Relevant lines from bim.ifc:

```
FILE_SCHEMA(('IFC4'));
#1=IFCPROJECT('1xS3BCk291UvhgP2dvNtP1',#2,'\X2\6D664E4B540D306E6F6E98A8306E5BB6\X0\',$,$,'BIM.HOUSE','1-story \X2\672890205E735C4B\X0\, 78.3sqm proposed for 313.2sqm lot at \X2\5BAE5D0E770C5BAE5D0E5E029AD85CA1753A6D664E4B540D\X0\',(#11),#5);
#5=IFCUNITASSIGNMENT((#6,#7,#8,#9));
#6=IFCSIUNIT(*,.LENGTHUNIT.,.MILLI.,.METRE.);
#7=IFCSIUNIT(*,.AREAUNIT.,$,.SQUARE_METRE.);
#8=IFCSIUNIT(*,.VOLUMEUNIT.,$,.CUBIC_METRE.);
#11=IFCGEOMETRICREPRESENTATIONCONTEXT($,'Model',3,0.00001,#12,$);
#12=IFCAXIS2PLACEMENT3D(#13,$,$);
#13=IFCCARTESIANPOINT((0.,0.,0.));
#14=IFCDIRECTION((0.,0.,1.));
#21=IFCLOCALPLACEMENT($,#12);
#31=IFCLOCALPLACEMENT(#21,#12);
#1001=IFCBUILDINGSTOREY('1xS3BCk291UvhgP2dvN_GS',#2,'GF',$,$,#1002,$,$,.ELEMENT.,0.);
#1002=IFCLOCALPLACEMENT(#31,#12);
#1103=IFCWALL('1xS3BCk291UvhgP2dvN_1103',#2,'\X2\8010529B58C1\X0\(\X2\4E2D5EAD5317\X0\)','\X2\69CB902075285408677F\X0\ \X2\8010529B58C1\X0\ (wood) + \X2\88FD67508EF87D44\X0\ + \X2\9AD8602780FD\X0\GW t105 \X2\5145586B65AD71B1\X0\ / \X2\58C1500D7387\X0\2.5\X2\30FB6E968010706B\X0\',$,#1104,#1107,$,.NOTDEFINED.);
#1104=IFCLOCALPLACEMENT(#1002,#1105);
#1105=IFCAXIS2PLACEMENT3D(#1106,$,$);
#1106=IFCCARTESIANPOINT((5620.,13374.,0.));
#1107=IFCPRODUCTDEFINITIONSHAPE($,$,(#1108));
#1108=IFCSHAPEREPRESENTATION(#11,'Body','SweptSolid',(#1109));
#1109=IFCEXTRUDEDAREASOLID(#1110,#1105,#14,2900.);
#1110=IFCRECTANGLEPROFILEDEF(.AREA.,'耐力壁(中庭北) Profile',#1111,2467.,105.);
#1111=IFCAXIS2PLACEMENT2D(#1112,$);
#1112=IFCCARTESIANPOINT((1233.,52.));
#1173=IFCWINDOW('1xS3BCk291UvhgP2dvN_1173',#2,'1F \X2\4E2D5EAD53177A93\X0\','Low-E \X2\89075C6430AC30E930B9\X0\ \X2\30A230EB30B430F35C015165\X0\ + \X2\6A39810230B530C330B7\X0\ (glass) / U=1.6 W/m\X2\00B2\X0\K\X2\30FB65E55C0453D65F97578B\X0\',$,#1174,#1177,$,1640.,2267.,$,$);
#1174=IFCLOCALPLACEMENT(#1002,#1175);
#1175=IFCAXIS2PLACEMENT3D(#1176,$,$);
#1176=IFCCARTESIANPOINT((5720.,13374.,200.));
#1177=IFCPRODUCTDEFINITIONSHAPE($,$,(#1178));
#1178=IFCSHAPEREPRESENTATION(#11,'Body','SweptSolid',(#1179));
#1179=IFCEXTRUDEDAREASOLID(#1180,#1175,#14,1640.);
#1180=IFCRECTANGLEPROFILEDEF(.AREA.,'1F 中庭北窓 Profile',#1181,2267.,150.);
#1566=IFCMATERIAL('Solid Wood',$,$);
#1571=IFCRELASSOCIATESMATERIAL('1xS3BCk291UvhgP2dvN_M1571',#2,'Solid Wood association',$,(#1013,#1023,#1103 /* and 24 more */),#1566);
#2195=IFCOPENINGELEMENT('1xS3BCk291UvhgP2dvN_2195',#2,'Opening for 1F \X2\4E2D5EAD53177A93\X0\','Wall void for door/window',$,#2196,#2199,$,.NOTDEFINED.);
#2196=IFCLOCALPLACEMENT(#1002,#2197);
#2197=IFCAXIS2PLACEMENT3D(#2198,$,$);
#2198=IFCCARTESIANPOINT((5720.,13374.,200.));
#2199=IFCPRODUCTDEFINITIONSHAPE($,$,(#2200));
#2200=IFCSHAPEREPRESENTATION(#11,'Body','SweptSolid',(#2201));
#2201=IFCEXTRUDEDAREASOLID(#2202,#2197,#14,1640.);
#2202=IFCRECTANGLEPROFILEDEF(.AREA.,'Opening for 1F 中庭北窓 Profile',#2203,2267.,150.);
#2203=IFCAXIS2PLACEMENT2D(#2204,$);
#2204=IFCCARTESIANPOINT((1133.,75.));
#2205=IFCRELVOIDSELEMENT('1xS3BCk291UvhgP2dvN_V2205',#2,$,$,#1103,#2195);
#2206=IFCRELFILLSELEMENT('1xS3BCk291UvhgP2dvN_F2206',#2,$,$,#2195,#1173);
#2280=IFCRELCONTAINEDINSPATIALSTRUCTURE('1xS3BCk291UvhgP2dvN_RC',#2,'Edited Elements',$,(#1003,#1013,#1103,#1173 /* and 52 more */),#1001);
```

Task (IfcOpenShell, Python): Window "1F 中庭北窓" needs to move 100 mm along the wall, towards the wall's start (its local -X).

```python
import ifcopenshell
import ifcopenshell.api.geometry
import ifcopenshell.util.placement

model = ifcopenshell.open("bim.ifc")

window = model.by_guid("1xS3BCk291UvhgP2dvN_1173")
opening = window.FillsVoids[0].RelatingOpeningElement
wall = opening.VoidsElements[0].RelatingBuildingElement

wall_matrix = ifcopenshell.util.placement.get_local_placement(wall.ObjectPlacement)
shift = wall_matrix[:3, 0] * -100.0
before = ifcopenshell.util.placement.get_local_placement(window.ObjectPlacement)[:3, 3].copy()

# The window is not placed relative to its opening, so move both.
for product in (opening, window):
    matrix = ifcopenshell.util.placement.get_local_placement(product.ObjectPlacement)
    matrix[:3, 3] += shift
    ifcopenshell.api.geometry.edit_object_placement(model, product=product, matrix=matrix, is_si=False)

after = ifcopenshell.util.placement.get_local_placement(window.ObjectPlacement)[:3, 3]
print("window moved by", (after - before).round(3) + 0.0)

model.write("bim_rev.ifc")
```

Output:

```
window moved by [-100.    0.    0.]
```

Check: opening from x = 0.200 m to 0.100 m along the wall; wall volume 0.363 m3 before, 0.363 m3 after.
